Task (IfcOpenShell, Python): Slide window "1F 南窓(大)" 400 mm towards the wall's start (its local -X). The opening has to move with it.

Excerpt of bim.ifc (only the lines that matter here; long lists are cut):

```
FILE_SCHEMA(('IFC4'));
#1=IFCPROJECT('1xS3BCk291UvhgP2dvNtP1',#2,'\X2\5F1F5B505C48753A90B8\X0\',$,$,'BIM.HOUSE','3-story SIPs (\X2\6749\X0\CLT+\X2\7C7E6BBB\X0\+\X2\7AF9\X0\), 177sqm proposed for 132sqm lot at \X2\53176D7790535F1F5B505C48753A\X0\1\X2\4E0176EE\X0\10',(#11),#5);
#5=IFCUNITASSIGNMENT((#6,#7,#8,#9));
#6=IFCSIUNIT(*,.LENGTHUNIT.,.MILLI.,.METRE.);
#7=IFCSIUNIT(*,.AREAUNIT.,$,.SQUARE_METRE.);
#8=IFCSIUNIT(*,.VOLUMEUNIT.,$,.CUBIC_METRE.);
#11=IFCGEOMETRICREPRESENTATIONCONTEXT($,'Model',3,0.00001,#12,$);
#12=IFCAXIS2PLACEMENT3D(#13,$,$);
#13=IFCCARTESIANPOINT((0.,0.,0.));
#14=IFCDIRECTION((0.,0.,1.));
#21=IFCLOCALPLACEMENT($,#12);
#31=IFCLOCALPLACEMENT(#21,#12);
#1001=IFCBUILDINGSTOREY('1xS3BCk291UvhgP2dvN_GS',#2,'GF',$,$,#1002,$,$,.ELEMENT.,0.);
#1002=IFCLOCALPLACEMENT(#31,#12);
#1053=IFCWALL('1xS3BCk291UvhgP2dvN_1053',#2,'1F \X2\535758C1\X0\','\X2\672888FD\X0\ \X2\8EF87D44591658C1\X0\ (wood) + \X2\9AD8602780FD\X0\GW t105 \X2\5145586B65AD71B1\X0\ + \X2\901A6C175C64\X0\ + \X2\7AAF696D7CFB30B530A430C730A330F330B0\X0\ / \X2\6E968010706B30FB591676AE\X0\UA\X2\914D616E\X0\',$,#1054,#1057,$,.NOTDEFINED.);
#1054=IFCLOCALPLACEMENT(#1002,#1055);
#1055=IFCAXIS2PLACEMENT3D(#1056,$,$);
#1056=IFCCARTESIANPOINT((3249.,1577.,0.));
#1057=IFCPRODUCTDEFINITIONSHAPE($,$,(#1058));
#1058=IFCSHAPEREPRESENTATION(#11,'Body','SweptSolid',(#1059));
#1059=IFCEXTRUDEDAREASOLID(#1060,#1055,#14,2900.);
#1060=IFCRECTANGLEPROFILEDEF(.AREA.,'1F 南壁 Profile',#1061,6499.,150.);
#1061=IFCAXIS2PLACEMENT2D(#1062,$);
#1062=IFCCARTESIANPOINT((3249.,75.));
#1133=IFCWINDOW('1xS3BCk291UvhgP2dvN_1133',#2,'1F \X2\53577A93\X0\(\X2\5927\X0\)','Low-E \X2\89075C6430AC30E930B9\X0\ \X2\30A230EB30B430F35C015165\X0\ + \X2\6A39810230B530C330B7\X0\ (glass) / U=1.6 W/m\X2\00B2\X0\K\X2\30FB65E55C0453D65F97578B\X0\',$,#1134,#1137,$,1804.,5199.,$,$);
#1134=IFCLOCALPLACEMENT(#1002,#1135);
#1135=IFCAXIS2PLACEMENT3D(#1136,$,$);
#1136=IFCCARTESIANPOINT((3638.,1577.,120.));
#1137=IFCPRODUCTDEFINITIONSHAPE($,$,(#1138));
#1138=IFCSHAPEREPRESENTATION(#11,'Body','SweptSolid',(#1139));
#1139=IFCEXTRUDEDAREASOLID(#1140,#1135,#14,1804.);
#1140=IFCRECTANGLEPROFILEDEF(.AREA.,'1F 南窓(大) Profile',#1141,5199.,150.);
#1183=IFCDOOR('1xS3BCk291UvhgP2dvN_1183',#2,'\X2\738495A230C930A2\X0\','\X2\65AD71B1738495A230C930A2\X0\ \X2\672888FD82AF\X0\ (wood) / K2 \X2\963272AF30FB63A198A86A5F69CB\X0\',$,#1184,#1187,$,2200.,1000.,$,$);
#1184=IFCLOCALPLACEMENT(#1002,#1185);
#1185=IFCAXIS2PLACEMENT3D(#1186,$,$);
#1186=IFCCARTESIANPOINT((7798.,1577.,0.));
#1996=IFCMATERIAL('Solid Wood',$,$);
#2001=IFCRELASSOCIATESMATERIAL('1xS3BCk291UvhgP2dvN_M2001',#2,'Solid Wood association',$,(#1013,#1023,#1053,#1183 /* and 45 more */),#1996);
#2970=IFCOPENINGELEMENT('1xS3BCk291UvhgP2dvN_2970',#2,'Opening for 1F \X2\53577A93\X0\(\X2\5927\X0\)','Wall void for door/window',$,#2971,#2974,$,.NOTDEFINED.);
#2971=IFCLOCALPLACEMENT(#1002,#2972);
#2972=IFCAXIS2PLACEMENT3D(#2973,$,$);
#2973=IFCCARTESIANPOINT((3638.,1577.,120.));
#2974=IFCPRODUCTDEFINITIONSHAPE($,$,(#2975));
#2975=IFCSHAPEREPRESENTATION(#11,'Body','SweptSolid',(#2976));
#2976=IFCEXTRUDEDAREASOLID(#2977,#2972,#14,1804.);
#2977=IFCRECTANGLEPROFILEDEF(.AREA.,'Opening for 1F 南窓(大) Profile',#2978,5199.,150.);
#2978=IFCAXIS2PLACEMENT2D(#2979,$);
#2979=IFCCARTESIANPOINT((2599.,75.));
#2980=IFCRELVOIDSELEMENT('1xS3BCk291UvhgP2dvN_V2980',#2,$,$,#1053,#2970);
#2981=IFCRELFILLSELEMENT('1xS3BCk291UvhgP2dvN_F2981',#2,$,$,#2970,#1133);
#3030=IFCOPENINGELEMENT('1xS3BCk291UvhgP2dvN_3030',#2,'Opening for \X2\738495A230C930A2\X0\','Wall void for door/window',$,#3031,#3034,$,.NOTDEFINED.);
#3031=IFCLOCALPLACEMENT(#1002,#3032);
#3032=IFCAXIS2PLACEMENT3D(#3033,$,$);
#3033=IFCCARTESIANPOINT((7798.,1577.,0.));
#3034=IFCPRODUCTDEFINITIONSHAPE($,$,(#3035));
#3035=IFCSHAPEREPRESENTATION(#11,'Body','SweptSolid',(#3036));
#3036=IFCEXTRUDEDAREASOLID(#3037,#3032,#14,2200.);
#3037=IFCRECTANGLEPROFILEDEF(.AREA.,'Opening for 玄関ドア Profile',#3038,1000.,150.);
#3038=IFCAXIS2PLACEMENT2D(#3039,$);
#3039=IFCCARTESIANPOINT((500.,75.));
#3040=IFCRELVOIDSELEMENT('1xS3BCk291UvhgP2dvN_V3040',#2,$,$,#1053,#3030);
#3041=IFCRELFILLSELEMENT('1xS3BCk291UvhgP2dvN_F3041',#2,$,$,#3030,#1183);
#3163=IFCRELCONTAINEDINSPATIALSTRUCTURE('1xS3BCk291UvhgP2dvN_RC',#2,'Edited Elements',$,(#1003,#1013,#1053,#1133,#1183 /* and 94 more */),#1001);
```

```python
import ifcopenshell
import ifcopenshell.api.geometry
import ifcopenshell.util.placement
import ifcopenshell.util.unit

model = ifcopenshell.open("bim.ifc")
unit_scale = ifcopenshell.util.unit.calculate_unit_scale(model)

window = model.by_id(1133)
opening = window.FillsVoids[0].RelatingOpeningElement
wall = opening.VoidsElements[0].RelatingBuildingElement

wall_matrix = ifcopenshell.util.placement.get_local_placement(wall.ObjectPlacement)
shift = wall_matrix[:3, 0] * -0.4 / unit_scale
before = ifcopenshell.util.placement.get_local_placement(window.ObjectPlacement)[:3, 3].copy()

# The window is not placed relative to its opening, so move both.
for product in (opening, window):
    matrix = ifcopenshell.util.placement.get_local_placement(product.ObjectPlacement)
    matrix[:3, 3] += shift
    ifcopenshell.api.geometry.edit_object_placement(model, product=product, matrix=matrix, is_si=False)

after = ifcopenshell.util.placement.get_local_placement(window.ObjectPlacement)[:3, 3]
print("window moved by", (after - before).round(3) + 0.0)

model.write("bim_edited.ifc")
```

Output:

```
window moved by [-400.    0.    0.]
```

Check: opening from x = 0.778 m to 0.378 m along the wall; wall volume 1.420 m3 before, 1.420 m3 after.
